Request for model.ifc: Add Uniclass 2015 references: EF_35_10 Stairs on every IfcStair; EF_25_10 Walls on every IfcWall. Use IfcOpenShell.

First a look at what the model holds.

```python
import ifcopenshell

model = ifcopenshell.open("model.ifc")
print(model.schema)
print("classifications:", [c.Name for c in model.by_type("IfcClassification")])
for ifc_class in ("IfcDoor", "IfcRoof", "IfcStair", "IfcWall", "IfcWindow"):
    print(ifc_class, len(model.by_type(ifc_class)))
```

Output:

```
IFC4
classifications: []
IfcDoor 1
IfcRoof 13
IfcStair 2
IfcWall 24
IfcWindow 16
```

```python
import ifcopenshell
import ifcopenshell.api.classification

model = ifcopenshell.open("model.ifc")

system = ifcopenshell.api.classification.add_classification(model, classification="Uniclass 2015")

codes = {
    "IfcStair": ("EF_35_10", "Stairs"),
    "IfcWall": ("EF_25_10", "Walls"),
}
for ifc_class, (code, name) in codes.items():
    products = model.by_type(ifc_class)
    ifcopenshell.api.classification.add_reference(
        model, products=products, classification=system, identification=code, name=name
    )
    print(code, len(products))

model.write("model_updated.ifc")
```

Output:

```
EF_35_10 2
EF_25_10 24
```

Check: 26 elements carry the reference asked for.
